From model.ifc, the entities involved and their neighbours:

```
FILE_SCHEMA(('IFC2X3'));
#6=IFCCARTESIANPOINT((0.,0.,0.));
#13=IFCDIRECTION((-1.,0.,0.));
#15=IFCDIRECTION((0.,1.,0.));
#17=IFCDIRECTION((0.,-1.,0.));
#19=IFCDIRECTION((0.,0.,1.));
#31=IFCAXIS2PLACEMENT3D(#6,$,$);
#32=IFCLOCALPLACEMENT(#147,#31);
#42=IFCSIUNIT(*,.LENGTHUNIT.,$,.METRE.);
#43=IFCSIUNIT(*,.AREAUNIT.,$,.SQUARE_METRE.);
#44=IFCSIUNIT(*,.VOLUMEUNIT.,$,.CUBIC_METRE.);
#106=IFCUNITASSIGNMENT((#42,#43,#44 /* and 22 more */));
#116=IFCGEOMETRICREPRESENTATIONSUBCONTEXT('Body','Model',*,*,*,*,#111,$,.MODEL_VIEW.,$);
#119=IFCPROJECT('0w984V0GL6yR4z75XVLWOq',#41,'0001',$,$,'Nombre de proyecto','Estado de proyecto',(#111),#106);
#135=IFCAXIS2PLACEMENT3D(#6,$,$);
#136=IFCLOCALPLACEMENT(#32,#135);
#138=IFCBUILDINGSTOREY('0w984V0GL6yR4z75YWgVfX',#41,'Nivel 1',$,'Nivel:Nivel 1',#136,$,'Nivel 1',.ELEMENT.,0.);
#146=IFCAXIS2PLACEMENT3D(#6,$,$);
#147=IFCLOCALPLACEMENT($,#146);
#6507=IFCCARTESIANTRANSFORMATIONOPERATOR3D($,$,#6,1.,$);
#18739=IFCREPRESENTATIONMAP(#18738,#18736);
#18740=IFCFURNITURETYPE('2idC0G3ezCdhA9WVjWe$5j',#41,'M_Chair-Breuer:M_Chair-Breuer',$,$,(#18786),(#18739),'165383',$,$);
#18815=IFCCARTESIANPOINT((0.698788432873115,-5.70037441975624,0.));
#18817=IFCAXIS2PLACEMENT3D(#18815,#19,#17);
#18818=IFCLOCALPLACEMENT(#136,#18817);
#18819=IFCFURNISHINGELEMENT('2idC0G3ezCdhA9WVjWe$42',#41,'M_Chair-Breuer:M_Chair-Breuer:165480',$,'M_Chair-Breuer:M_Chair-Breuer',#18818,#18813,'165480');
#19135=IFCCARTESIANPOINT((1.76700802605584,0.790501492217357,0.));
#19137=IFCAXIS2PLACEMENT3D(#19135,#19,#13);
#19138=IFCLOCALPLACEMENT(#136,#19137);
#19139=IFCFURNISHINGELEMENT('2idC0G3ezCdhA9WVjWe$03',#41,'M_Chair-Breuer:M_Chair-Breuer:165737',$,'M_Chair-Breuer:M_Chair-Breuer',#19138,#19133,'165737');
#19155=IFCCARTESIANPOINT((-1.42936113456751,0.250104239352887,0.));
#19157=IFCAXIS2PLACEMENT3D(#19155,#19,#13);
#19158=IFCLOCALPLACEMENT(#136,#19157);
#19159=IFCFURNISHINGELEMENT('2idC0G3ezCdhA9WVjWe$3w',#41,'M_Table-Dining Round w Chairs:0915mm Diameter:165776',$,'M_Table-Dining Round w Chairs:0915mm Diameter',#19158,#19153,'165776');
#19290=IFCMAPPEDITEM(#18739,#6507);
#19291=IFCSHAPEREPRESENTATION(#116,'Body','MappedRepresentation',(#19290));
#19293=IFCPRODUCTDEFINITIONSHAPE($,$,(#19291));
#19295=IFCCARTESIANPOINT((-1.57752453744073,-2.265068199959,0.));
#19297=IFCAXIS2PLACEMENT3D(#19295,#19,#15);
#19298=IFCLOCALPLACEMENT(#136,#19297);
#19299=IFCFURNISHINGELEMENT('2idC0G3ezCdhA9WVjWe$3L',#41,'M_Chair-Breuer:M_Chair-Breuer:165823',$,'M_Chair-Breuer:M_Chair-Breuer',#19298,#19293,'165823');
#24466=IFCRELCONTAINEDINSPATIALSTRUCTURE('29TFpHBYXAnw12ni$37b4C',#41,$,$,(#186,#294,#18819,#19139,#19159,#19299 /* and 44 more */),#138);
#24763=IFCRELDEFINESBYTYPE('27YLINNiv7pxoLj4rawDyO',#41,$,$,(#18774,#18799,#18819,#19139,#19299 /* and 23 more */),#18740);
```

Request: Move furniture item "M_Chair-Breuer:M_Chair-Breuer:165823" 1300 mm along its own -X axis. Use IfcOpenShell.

```python
import ifcopenshell
import ifcopenshell.api.geometry
import ifcopenshell.util.placement
import ifcopenshell.util.unit

model = ifcopenshell.open("model.ifc")
unit_scale = ifcopenshell.util.unit.calculate_unit_scale(model)

item = model.by_id(19299)
matrix = ifcopenshell.util.placement.get_local_placement(item.ObjectPlacement)
matrix[:3, 3] -= matrix[:3, 0] * 1.3 / unit_scale
ifcopenshell.api.geometry.edit_object_placement(model, product=item, matrix=matrix, is_si=False)

print(ifcopenshell.util.placement.get_local_placement(item.ObjectPlacement).round(3) + 0.0)

model.write("model_v2.ifc")
```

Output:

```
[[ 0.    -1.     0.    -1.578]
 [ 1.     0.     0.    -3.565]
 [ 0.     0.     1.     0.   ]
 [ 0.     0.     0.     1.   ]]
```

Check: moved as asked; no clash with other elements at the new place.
